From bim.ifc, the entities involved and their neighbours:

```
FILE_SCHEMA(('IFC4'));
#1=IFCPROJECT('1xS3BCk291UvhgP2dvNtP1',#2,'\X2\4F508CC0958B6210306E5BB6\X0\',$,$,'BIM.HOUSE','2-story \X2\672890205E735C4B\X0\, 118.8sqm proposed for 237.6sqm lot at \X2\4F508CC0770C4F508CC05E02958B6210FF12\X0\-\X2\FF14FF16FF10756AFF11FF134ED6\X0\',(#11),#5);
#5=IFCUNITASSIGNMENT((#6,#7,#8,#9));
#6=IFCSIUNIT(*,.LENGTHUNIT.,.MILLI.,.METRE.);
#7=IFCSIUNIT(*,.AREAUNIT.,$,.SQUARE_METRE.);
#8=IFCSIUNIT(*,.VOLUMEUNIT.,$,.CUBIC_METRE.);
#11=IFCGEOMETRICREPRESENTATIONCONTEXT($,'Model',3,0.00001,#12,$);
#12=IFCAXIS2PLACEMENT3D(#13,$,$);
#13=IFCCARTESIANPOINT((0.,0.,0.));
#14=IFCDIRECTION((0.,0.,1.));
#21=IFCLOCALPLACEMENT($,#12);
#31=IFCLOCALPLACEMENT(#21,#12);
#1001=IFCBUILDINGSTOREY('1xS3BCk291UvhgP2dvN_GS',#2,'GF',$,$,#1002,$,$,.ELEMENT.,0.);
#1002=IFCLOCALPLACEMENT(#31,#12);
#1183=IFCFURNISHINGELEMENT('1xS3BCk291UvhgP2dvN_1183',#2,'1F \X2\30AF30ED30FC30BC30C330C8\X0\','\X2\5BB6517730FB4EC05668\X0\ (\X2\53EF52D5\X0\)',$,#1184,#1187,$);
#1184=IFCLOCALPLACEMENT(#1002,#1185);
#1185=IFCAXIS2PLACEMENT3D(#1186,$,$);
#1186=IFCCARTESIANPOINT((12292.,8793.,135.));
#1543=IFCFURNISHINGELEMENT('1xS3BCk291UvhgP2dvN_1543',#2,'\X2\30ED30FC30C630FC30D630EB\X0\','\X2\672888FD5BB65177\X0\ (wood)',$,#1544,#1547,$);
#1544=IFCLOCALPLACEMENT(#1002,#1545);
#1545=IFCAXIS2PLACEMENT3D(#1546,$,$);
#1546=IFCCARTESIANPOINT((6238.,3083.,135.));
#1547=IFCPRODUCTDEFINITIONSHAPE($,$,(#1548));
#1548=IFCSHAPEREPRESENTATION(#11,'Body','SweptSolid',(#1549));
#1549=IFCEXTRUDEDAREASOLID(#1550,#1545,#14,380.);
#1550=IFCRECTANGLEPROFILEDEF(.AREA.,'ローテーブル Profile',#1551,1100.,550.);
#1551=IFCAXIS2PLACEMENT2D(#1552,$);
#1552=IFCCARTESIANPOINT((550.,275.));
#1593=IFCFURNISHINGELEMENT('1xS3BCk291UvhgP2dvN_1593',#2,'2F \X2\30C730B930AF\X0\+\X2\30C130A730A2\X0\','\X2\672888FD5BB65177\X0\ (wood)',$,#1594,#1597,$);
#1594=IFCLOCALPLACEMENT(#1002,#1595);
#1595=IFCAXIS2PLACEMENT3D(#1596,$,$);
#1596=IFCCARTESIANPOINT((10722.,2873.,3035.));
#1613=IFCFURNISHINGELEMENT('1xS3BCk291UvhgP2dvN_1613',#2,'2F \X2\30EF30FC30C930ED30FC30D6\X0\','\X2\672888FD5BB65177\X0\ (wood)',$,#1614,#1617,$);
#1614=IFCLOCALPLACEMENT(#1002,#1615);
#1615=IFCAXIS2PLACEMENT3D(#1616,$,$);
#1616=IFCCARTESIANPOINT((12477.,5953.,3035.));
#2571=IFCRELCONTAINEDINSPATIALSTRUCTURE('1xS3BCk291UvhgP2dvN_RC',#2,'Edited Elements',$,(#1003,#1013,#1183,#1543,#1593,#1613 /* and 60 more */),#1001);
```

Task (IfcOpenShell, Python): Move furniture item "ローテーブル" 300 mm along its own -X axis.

```python
import ifcopenshell
import ifcopenshell.api.geometry
import ifcopenshell.util.placement

model = ifcopenshell.open("bim.ifc")

item = model.by_guid("1xS3BCk291UvhgP2dvN_1543")
matrix = ifcopenshell.util.placement.get_local_placement(item.ObjectPlacement)
matrix[:3, 3] -= matrix[:3, 0] * 300.0
ifcopenshell.api.geometry.edit_object_placement(model, product=item, matrix=matrix, is_si=False)

print(ifcopenshell.util.placement.get_local_placement(item.ObjectPlacement).round(3) + 0.0)

model.write("bim_updated.ifc")
```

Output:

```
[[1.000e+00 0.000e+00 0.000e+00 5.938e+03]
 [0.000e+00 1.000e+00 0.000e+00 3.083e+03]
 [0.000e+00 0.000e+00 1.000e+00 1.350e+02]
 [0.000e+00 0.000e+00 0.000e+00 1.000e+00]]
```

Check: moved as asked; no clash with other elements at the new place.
